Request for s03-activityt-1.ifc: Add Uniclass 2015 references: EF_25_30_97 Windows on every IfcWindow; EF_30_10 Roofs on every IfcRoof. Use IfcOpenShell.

First a look at what the model holds.

```python
import ifcopenshell

model = ifcopenshell.open("s03-activityt-1.ifc")
print(model.schema)
print("classifications:", [c.Name for c in model.by_type("IfcClassification")])
for ifc_class in ("IfcDoor", "IfcRoof", "IfcStair", "IfcWall", "IfcWindow"):
    print(ifc_class, len(model.by_type(ifc_class)))
```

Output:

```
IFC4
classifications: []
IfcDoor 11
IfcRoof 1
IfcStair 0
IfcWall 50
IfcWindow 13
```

```python
import ifcopenshell
import ifcopenshell.api.classification

model = ifcopenshell.open("s03-activityt-1.ifc")

system = ifcopenshell.api.classification.add_classification(model, classification="Uniclass 2015")

codes = {
    "IfcWindow": ("EF_25_30_97", "Windows"),
    "IfcRoof": ("EF_30_10", "Roofs"),
}
for ifc_class, (code, name) in codes.items():
    products = model.by_type(ifc_class)
    ifcopenshell.api.classification.add_reference(
        model, products=products, classification=system, identification=code, name=name
    )
    print(code, len(products))

model.write("s03-activityt-1-out.ifc")
```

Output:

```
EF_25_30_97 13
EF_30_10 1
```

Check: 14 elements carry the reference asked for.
